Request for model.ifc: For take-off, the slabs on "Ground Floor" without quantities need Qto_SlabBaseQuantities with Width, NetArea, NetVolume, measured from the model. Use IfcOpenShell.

First a look at what the model holds.

```python
import ifcopenshell
import ifcopenshell.util.element
import ifcopenshell.util.unit

model = ifcopenshell.open("model.ifc")
print(model.schema)
for unit_type in ("LENGTHUNIT", "AREAUNIT", "VOLUMEUNIT"):
    print(unit_type, ifcopenshell.util.unit.calculate_unit_scale(model, unit_type))
storey = next(s for s in model.by_type("IfcBuildingStorey") if s.Name == "Ground Floor")
slabs = [e for e in ifcopenshell.util.element.get_decomposition(storey) if e.is_a("IfcSlab")]
for e in sorted(slabs, key=lambda e: e.id()):
    print(e.id(), e.is_a(), e.Name, list(ifcopenshell.util.element.get_psets(e, qtos_only=True)), sep=" | ")
```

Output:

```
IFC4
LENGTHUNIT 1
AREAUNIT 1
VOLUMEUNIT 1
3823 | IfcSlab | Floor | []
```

```python
import ifcopenshell
import ifcopenshell.api.pset
import ifcopenshell.geom
import ifcopenshell.util.element
import ifcopenshell.util.shape
import ifcopenshell.util.unit

model = ifcopenshell.open("model.ifc")
unit_scale = ifcopenshell.util.unit.calculate_unit_scale(model)
area_scale = ifcopenshell.util.unit.calculate_unit_scale(model, "AREAUNIT")
volume_scale = ifcopenshell.util.unit.calculate_unit_scale(model, "VOLUMEUNIT")
settings = ifcopenshell.geom.settings()

storey = next(s for s in model.by_type("IfcBuildingStorey") if s.Name == "Ground Floor")
slabs = [e for e in ifcopenshell.util.element.get_decomposition(storey) if e.is_a("IfcSlab")]

for e in sorted(slabs, key=lambda e: e.id()):
    if ifcopenshell.util.element.get_psets(e, qtos_only=True, should_inherit=False):
        continue
    # Geometry comes back in metres, in the element's own axes.
    shape = ifcopenshell.geom.create_shape(settings, e)
    values = {
        "Width": ifcopenshell.util.shape.get_z(shape.geometry) / unit_scale,
        "NetArea": ifcopenshell.util.shape.get_footprint_area(shape.geometry) / area_scale,
        "NetVolume": ifcopenshell.util.shape.get_volume(shape.geometry) / volume_scale,
    }
    qto = ifcopenshell.api.pset.add_qto(model, product=e, name="Qto_SlabBaseQuantities")
    ifcopenshell.api.pset.edit_qto(model, qto=qto, properties=values)
    print(e.id(), {k: round(v, 3) for k, v in values.items()})

model.write("model_v2.ifc")
```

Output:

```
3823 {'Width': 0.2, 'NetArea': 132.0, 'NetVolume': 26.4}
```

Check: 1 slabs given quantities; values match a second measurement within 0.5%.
